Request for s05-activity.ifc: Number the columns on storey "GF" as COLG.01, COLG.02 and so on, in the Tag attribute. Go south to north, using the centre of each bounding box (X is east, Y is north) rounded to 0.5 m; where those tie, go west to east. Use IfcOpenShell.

First a look at what the model holds.

```python
import ifcopenshell
import ifcopenshell.util.element
import ifcopenshell.util.placement

model = ifcopenshell.open("s05-activity.ifc")
print(model.schema)
storey = next(s for s in model.by_type("IfcBuildingStorey") if s.Name == "GF")
columns = [e for e in ifcopenshell.util.element.get_decomposition(storey) if e.is_a("IfcColumn")]
for e in sorted(columns, key=lambda e: e.id()):
    origin = ifcopenshell.util.placement.get_local_placement(e.ObjectPlacement)[:3, 3]
    print(e.id(), e.Tag, e.Name, origin.round(2) + 0.0, sep=" | ")
```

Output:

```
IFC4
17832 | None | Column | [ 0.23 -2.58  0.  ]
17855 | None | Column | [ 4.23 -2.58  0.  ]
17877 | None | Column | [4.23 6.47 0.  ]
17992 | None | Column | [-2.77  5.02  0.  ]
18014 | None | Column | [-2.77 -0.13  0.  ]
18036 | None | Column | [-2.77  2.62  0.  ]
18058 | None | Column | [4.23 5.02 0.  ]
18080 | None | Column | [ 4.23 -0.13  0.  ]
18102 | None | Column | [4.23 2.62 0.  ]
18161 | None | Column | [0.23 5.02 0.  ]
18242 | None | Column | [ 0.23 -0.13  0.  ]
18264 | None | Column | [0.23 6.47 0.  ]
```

```python
import ifcopenshell
import ifcopenshell.geom
import ifcopenshell.util.element
import ifcopenshell.util.shape

model = ifcopenshell.open("s05-activity.ifc")
settings = ifcopenshell.geom.settings()
settings.set("use-world-coords", True)


def centre(element):
    shape = ifcopenshell.geom.create_shape(settings, element)
    return ifcopenshell.util.shape.get_bbox_centroid(shape.geometry)


storey = next(s for s in model.by_type("IfcBuildingStorey") if s.Name == "GF")
columns = [e for e in ifcopenshell.util.element.get_decomposition(storey) if e.is_a("IfcColumn")]

# Insertion points can sit at a corner or the storey origin, so sort by the geometry (in metres).
centres = {e: centre(e) for e in columns}
columns.sort(key=lambda e: (round(centres[e][1] / 0.5), centres[e][0]))

for i, e in enumerate(columns, start=1):
    number = f"COLG.{i:02d}"
    e.Tag = number
    print(e.id(), number)

model.write("s05-activity_edited.ifc")
```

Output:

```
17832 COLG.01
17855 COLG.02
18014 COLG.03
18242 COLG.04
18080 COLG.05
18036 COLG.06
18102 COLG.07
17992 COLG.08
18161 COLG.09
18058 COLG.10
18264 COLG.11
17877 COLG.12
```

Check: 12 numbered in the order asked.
